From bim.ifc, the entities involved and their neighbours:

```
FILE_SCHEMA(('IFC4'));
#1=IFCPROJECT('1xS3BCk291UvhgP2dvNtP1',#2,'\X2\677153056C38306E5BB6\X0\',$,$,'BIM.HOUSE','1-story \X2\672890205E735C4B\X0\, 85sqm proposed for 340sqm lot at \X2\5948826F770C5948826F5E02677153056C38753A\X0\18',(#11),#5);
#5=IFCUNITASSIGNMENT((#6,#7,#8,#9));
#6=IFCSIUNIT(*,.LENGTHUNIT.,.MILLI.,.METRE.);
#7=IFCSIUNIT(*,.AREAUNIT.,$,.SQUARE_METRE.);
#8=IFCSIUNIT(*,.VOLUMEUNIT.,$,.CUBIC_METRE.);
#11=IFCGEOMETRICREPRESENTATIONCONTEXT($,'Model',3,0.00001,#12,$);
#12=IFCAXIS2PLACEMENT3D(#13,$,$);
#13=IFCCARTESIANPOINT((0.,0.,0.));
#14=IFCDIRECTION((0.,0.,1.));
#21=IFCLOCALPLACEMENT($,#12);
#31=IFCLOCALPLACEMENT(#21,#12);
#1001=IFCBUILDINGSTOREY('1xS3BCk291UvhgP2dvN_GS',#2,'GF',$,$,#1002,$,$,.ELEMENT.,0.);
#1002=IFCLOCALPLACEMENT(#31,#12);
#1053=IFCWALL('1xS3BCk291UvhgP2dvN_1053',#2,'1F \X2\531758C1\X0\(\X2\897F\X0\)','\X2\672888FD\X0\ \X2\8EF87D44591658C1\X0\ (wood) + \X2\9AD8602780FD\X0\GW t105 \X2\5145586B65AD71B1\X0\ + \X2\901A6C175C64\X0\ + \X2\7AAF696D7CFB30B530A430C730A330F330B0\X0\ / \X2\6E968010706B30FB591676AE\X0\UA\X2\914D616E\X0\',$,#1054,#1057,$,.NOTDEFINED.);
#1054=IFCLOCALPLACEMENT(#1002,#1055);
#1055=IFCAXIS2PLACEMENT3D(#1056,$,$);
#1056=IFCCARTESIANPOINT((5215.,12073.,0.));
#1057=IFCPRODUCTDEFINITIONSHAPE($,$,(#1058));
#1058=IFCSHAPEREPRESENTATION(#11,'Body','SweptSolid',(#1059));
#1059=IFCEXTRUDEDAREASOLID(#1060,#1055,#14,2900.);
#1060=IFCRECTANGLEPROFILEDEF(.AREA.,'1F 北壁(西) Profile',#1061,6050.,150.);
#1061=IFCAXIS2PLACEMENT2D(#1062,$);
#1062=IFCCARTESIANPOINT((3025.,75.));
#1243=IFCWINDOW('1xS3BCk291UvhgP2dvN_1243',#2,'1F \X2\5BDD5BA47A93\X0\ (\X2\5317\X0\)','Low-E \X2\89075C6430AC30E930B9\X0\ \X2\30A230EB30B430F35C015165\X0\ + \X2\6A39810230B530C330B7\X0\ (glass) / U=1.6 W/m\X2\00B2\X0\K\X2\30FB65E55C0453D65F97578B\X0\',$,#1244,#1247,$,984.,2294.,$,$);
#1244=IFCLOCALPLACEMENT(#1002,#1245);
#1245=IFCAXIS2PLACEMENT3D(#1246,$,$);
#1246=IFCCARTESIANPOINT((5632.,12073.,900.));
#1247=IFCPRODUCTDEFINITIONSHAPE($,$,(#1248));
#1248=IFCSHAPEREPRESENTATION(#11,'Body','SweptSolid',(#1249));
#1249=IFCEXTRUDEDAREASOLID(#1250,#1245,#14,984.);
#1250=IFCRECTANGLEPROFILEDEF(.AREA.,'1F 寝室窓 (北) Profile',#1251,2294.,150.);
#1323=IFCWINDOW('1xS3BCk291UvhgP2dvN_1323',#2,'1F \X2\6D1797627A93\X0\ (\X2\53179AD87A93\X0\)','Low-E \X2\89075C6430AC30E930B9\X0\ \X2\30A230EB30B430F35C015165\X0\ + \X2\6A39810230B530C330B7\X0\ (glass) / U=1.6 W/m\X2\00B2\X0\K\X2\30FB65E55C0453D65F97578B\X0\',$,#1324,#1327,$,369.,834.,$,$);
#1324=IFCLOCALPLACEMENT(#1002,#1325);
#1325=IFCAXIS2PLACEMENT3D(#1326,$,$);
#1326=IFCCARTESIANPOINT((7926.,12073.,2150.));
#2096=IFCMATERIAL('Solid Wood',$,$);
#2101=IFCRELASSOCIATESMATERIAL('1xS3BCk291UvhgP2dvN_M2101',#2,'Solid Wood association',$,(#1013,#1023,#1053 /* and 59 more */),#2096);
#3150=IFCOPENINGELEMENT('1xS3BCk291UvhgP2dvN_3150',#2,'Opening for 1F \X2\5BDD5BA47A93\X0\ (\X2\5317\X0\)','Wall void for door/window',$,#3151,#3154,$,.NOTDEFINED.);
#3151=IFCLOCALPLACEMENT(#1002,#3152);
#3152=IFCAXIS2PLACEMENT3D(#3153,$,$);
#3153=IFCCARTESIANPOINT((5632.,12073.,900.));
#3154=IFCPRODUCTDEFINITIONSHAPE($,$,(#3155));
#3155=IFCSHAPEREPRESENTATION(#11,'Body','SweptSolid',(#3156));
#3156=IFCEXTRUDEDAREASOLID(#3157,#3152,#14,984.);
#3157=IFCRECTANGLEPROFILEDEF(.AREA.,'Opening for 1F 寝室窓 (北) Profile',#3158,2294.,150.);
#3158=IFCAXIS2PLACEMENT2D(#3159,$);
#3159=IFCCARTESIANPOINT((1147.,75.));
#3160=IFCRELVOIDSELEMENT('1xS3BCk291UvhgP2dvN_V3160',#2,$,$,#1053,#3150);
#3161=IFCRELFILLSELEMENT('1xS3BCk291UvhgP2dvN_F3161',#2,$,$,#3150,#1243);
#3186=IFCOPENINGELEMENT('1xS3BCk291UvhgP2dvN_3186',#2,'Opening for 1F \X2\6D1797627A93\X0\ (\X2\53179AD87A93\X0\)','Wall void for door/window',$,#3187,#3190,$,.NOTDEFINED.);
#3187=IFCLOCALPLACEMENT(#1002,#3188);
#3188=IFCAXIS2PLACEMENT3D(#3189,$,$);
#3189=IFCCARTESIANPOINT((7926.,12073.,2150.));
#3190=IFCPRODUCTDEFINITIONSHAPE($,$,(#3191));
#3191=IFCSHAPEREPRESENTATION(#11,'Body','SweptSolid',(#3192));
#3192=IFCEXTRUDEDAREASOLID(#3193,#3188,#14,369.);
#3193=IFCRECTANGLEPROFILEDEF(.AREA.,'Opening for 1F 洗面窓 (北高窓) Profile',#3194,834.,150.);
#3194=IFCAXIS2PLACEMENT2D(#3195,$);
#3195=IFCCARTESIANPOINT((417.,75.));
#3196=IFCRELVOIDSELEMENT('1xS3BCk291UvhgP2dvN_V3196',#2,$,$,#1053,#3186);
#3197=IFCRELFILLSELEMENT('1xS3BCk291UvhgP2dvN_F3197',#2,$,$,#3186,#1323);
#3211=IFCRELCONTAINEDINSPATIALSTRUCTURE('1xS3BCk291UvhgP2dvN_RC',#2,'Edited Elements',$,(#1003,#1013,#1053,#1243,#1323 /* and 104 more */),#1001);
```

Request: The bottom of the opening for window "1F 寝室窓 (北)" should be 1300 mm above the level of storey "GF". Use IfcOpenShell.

```python
import numpy as np
import ifcopenshell
import ifcopenshell.api.geometry
import ifcopenshell.geom
import ifcopenshell.util.element
import ifcopenshell.util.placement
import ifcopenshell.util.shape
import ifcopenshell.util.unit

model = ifcopenshell.open("bim.ifc")
unit_scale = ifcopenshell.util.unit.calculate_unit_scale(model)

window = model.by_guid("1xS3BCk291UvhgP2dvN_1243")
opening = window.FillsVoids[0].RelatingOpeningElement
storey = ifcopenshell.util.element.get_container(window, ifc_class="IfcBuildingStorey")
level = ifcopenshell.util.placement.get_local_placement(storey.ObjectPlacement)[2, 3]

# The opening's origin need not be at the sill, so measure its lowest point.
shape = ifcopenshell.geom.create_shape(ifcopenshell.geom.settings(), opening)
bottom = ifcopenshell.util.shape.get_shape_bottom_elevation(shape, shape.geometry) / unit_scale
dz = level + 1300.0 - bottom

shift = np.array([0.0, 0.0, dz])
# The window is not placed relative to its opening, so move both.
for product in (opening, window):
    matrix = ifcopenshell.util.placement.get_local_placement(product.ObjectPlacement)
    matrix[:3, 3] += shift
    ifcopenshell.api.geometry.edit_object_placement(model, product=product, matrix=matrix, is_si=False)

print(f"moved by {dz * unit_scale:+.3f} m")

model.write("bim-out.ifc")
```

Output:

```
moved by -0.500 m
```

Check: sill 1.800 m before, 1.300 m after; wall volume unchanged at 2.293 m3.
